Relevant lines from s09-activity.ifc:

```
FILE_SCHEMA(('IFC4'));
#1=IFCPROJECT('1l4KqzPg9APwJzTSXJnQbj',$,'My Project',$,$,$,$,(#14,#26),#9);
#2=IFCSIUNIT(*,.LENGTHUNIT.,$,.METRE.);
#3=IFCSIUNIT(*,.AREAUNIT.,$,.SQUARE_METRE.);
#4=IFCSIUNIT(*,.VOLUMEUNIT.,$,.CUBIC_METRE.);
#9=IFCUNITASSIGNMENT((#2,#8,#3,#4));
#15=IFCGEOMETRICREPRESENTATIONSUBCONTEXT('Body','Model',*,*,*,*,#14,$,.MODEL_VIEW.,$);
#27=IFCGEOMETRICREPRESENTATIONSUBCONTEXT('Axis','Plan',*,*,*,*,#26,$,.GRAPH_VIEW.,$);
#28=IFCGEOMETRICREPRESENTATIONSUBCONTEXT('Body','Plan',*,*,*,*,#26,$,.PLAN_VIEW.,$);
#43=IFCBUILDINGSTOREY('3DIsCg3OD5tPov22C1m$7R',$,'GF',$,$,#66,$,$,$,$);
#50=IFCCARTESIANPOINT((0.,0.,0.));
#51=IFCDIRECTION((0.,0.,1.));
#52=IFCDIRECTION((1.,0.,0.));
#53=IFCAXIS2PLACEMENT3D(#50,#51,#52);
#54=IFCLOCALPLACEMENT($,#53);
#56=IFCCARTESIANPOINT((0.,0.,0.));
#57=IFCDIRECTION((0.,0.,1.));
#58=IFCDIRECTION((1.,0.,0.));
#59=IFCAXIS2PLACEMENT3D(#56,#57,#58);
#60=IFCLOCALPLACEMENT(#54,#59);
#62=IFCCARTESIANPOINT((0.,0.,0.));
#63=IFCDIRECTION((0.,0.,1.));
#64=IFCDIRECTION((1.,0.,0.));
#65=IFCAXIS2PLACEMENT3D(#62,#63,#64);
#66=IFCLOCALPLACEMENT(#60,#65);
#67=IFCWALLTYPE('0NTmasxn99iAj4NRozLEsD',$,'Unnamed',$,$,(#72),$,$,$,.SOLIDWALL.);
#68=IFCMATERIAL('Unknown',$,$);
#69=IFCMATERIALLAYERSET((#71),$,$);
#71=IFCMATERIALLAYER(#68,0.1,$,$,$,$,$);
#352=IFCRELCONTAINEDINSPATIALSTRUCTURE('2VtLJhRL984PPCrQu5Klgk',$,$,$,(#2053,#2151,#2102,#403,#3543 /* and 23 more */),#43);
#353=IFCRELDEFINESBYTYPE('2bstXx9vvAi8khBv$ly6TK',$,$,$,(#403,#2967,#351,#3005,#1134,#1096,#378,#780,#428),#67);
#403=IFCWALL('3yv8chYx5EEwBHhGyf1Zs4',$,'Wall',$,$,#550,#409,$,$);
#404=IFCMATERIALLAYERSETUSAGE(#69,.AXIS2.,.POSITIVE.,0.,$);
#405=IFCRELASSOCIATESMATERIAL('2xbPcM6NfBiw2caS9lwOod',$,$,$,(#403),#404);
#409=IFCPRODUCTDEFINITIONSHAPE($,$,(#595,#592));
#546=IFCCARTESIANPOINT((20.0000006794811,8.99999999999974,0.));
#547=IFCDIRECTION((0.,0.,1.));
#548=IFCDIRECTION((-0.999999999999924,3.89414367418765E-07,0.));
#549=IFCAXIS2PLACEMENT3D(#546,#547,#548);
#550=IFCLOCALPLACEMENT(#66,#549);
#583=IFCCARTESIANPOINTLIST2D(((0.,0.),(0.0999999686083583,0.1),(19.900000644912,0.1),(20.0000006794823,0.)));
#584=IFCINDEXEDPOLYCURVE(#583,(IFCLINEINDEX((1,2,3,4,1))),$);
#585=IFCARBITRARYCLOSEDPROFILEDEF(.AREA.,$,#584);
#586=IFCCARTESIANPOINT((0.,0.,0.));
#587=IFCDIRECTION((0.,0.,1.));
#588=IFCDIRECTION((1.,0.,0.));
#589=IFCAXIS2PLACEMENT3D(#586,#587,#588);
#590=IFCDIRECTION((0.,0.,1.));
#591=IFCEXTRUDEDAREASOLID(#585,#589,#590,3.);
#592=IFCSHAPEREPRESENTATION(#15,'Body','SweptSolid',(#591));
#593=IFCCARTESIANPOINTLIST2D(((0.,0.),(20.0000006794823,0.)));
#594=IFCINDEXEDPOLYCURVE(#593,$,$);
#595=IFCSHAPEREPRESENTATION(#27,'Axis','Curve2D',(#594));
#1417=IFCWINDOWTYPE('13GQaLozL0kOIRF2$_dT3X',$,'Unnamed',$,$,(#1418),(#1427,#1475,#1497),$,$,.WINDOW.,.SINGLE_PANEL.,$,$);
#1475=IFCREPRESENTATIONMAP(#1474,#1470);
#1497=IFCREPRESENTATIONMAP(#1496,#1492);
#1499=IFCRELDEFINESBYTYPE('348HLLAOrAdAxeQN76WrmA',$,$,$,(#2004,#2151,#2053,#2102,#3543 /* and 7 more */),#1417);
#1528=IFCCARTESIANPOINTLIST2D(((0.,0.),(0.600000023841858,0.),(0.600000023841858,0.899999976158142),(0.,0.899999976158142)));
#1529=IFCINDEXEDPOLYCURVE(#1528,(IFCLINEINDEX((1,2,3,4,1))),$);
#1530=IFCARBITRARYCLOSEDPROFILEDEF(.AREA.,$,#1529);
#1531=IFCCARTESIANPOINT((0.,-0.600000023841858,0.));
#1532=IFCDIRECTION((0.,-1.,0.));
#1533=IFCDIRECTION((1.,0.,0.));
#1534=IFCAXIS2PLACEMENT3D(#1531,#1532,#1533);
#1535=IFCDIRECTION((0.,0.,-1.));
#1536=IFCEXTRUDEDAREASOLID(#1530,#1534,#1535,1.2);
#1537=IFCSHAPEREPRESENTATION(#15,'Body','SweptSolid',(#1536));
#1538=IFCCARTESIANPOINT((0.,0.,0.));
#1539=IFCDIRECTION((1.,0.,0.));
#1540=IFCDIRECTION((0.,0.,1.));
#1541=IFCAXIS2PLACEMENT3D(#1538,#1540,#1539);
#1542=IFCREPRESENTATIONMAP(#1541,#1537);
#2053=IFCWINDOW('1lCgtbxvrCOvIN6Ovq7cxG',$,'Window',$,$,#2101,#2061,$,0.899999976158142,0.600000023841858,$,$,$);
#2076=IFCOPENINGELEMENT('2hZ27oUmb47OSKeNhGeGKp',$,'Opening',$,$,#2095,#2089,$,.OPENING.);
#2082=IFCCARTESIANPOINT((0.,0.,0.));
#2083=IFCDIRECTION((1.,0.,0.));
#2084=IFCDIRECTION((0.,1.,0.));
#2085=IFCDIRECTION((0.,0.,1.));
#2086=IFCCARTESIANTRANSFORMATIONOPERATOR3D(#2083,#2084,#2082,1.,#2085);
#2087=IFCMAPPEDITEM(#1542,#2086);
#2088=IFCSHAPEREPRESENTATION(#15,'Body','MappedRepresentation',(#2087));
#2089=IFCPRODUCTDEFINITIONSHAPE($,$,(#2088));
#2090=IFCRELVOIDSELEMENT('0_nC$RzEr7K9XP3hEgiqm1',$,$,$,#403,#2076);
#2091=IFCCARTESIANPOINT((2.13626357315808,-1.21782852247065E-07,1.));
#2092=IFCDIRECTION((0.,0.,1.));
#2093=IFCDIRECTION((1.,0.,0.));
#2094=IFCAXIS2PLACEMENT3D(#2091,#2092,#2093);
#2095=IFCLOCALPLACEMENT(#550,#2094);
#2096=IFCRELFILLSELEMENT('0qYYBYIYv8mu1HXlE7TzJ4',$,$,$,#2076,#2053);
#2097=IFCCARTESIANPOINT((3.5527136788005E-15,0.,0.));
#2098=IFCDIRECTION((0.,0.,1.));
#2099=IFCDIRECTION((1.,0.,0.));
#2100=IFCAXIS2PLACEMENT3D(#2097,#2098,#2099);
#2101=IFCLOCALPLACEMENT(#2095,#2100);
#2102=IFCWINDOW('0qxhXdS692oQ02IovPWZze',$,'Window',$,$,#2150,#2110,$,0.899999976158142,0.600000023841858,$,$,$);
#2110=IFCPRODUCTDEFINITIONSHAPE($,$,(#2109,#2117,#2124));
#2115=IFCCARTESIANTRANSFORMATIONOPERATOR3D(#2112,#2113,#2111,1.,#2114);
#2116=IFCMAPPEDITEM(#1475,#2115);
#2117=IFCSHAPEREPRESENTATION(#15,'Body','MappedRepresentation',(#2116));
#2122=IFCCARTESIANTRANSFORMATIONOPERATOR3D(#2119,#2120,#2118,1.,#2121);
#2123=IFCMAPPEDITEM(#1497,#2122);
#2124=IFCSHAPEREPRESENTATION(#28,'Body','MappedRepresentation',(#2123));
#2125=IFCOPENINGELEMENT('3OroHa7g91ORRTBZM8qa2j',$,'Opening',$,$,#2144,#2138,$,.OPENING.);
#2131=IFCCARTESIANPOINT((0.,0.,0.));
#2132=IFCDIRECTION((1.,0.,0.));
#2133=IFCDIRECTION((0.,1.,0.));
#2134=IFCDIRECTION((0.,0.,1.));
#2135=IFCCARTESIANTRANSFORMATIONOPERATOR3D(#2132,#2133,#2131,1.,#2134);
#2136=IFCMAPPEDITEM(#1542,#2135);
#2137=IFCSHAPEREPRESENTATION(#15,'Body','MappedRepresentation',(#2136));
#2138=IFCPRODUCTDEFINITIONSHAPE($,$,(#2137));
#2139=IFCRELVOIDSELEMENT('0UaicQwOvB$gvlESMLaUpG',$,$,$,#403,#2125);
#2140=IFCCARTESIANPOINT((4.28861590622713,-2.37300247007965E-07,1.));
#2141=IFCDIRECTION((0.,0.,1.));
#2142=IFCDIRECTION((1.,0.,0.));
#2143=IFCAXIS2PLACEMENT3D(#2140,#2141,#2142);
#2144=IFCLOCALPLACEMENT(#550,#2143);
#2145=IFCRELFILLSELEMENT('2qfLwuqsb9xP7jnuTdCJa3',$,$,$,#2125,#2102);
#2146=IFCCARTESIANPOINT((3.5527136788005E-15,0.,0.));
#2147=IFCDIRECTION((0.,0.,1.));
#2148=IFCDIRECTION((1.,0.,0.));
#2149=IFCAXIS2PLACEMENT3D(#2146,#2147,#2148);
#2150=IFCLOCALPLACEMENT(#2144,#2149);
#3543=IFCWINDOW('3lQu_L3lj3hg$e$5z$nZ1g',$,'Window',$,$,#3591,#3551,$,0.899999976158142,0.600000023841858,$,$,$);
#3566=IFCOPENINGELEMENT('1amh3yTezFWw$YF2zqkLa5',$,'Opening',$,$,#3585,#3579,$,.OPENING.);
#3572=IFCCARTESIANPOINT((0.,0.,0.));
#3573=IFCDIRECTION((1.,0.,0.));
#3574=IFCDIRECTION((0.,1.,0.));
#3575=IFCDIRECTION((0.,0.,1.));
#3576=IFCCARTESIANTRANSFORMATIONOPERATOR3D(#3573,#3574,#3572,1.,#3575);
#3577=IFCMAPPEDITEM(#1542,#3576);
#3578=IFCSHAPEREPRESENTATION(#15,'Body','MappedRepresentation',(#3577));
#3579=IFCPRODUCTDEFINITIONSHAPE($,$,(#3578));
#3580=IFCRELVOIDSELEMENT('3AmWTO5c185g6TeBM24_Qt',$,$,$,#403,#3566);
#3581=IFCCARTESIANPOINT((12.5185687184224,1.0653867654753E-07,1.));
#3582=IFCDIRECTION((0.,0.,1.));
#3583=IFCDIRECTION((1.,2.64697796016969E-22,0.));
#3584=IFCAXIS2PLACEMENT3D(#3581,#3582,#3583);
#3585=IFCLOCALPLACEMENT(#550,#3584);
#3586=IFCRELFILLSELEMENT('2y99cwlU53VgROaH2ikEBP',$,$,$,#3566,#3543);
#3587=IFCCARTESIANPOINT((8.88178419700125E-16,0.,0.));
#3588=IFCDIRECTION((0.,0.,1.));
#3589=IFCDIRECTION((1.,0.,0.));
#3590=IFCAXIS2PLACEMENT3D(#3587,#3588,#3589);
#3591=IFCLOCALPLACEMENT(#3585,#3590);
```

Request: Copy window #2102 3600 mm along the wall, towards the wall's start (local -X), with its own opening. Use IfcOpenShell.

```python
import ifcopenshell
import ifcopenshell.api.feature
import ifcopenshell.api.geometry
import ifcopenshell.api.root
import ifcopenshell.geom
import ifcopenshell.util.element
import ifcopenshell.util.placement
import ifcopenshell.util.shape

model = ifcopenshell.open("s09-activity.ifc")
settings = ifcopenshell.geom.settings()


def volume(element):
    """Net volume in cubic metres, openings subtracted."""
    shape = ifcopenshell.geom.create_shape(settings, element)
    return ifcopenshell.util.shape.get_volume(shape.geometry)


window = model.by_guid("0qxhXdS692oQ02IovPWZze")
opening = window.FillsVoids[0].RelatingOpeningElement
wall = opening.VoidsElements[0].RelatingBuildingElement
before = volume(wall)
shift = ifcopenshell.util.placement.get_local_placement(wall.ObjectPlacement)[:3, 0] * -3.6

# copy_class copies the void relationship, type, container and properties, but no geometry.
new_opening = ifcopenshell.api.root.copy_class(model, product=opening)
new_opening.Representation = ifcopenshell.util.element.copy_deep(
    model, opening.Representation, exclude=["IfcGeometricRepresentationContext", "IfcRepresentationMap"]
)
new_window = ifcopenshell.api.root.copy_class(model, product=window)
new_window.Representation = ifcopenshell.util.element.copy_deep(
    model, window.Representation, exclude=["IfcGeometricRepresentationContext", "IfcRepresentationMap"]
)
ifcopenshell.api.feature.add_filling(model, opening=new_opening, element=new_window)

for old, new in ((opening, new_opening), (window, new_window)):
    matrix = ifcopenshell.util.placement.get_local_placement(old.ObjectPlacement)
    matrix[:3, 3] += shift
    ifcopenshell.api.geometry.edit_object_placement(model, product=new, matrix=matrix, is_si=False)

after = volume(wall)

print(f"wall volume {before:.3f} -> {after:.3f} m3")

model.write("s09-activity_rev.ifc")
```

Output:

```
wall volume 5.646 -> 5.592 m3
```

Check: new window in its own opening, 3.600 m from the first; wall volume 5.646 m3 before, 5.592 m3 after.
